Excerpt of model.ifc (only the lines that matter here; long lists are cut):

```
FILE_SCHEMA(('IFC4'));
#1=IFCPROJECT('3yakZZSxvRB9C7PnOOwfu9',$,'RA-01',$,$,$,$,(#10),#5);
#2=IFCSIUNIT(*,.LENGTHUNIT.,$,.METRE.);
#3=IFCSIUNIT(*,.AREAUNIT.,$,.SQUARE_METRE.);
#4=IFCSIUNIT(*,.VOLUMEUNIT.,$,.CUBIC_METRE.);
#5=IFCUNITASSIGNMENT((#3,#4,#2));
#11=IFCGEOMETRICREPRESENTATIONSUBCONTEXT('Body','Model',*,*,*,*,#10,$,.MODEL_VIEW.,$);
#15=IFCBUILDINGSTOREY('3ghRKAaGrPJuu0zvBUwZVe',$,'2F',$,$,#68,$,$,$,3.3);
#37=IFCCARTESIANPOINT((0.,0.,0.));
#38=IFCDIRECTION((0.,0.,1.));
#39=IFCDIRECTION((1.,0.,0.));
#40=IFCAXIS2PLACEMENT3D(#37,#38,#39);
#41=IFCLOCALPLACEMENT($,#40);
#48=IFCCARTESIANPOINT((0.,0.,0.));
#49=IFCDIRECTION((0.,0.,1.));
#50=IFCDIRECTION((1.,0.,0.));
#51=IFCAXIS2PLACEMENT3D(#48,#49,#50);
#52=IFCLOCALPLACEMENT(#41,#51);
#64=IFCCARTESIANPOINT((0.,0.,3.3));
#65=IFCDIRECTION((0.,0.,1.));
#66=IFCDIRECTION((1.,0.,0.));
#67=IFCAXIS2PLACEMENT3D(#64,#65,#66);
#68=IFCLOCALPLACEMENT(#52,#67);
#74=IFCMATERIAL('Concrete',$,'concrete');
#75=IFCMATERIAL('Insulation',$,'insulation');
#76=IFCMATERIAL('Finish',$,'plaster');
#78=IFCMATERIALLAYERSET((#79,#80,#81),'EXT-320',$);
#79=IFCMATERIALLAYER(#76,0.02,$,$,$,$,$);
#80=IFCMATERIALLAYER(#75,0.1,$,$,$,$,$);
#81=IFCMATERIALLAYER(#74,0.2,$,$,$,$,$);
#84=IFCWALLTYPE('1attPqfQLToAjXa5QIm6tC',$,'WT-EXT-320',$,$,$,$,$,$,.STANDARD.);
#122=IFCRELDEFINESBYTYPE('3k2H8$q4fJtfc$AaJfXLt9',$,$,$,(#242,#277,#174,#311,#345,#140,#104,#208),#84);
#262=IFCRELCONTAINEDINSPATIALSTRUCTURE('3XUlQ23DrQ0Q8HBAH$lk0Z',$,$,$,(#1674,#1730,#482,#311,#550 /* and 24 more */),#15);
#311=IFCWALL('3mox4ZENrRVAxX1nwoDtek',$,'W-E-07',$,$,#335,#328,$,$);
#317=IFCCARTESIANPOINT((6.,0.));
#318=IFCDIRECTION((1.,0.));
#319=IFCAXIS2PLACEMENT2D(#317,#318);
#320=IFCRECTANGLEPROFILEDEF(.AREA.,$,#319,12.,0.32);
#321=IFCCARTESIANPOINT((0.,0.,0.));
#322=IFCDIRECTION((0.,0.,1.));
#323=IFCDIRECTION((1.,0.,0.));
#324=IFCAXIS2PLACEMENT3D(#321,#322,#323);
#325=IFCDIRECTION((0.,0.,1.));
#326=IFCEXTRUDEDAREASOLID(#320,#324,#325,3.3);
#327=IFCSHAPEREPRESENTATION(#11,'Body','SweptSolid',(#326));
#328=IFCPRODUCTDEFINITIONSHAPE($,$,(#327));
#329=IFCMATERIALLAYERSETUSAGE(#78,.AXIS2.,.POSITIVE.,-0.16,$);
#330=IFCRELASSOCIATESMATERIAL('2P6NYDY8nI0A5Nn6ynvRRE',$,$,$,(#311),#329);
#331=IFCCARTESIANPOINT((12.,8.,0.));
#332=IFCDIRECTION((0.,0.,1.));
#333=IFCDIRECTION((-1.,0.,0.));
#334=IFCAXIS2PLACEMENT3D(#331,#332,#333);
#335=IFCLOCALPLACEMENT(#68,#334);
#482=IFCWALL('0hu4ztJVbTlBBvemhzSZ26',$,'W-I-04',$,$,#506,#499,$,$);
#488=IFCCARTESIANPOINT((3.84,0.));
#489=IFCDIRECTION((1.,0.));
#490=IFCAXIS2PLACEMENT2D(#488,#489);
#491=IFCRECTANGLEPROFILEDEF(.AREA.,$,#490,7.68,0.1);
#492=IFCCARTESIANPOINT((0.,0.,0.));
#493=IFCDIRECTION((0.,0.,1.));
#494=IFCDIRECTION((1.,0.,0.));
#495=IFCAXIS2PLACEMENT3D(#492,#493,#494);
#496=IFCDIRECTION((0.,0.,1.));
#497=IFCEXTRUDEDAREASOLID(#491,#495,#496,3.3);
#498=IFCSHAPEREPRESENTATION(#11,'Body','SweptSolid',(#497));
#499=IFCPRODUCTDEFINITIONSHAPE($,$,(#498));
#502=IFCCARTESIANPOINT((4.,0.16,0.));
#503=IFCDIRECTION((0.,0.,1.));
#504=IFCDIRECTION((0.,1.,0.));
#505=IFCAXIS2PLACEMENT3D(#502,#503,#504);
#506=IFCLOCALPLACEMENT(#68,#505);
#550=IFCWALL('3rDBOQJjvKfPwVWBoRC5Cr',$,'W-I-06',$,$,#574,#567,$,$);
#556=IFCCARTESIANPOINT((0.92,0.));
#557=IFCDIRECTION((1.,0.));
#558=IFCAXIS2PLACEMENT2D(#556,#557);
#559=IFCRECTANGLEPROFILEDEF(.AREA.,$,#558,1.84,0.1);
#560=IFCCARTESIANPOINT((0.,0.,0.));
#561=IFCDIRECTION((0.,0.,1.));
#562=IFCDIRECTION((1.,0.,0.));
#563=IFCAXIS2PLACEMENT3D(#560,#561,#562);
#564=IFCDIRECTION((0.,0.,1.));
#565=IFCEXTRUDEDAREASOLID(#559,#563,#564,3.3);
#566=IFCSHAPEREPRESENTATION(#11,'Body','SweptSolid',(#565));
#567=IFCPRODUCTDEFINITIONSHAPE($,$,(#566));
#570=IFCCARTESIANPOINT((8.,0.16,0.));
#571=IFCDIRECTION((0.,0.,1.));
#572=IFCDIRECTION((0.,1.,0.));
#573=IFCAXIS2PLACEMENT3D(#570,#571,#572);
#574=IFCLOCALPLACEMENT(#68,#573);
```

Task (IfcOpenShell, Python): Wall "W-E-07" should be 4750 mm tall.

```python
import ifcopenshell
import ifcopenshell.geom
import ifcopenshell.util.representation
import ifcopenshell.util.shape

model = ifcopenshell.open("model.ifc")
settings = ifcopenshell.geom.settings()


def volume(element):
    """Net volume in cubic metres, openings subtracted."""
    shape = ifcopenshell.geom.create_shape(settings, element)
    return ifcopenshell.util.shape.get_volume(shape.geometry)


wall = model.by_guid("3mox4ZENrRVAxX1nwoDtek")
before = volume(wall)

body = ifcopenshell.util.representation.get_representation(wall, "Model", "Body")
solid = body.Items[0]
old_height = solid.Depth
solid.Depth = 4.75
after = volume(wall)

print(f"height {old_height:g} -> {solid.Depth:g}, volume {before:.3f} -> {after:.3f} m3")

model.write("model-out.ifc")
```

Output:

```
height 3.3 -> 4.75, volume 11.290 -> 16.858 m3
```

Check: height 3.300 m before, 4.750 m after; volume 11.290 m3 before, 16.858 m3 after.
